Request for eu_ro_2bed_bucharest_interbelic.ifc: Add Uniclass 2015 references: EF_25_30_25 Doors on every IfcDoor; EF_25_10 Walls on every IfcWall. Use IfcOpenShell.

First a look at what the model holds.

```python
import ifcopenshell

model = ifcopenshell.open("eu_ro_2bed_bucharest_interbelic.ifc")
print(model.schema)
print("classifications:", [c.Name for c in model.by_type("IfcClassification")])
for ifc_class in ("IfcDoor", "IfcRoof", "IfcStair", "IfcWall", "IfcWindow"):
    print(ifc_class, len(model.by_type(ifc_class)))
```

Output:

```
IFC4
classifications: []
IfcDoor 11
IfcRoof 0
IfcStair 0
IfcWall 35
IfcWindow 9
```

```python
import ifcopenshell
import ifcopenshell.api.classification

model = ifcopenshell.open("eu_ro_2bed_bucharest_interbelic.ifc")

system = ifcopenshell.api.classification.add_classification(model, classification="Uniclass 2015")

codes = {
    "IfcDoor": ("EF_25_30_25", "Doors"),
    "IfcWall": ("EF_25_10", "Walls"),
}
for ifc_class, (code, name) in codes.items():
    products = model.by_type(ifc_class)
    ifcopenshell.api.classification.add_reference(
        model, products=products, classification=system, identification=code, name=name
    )
    print(code, len(products))

model.write("eu_ro_2bed_bucharest_interbelic-out.ifc")
```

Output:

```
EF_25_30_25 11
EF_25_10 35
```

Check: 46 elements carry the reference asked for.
